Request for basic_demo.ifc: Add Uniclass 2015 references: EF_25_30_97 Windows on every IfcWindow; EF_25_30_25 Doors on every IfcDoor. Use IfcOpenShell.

First a look at what the model holds.

```python
import ifcopenshell

model = ifcopenshell.open("basic_demo.ifc")
print(model.schema)
print("classifications:", [c.Name for c in model.by_type("IfcClassification")])
for ifc_class in ("IfcDoor", "IfcRoof", "IfcStair", "IfcWall", "IfcWindow"):
    print(ifc_class, len(model.by_type(ifc_class)))
```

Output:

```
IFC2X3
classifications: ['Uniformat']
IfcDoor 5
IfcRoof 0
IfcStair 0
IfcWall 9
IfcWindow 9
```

```python
import ifcopenshell
import ifcopenshell.api.classification

model = ifcopenshell.open("basic_demo.ifc")

# IFC2X3 requires Source and Edition and has no link from the project to the system.
system = model.create_entity("IfcClassification", Source="NBS", Edition="2015", Name="Uniclass 2015")

codes = {
    "IfcWindow": ("EF_25_30_97", "Windows"),
    "IfcDoor": ("EF_25_30_25", "Doors"),
}
for ifc_class, (code, name) in codes.items():
    products = model.by_type(ifc_class)
    ifcopenshell.api.classification.add_reference(
        model, products=products, classification=system, identification=code, name=name
    )
    print(code, len(products))

model.write("basic_demo_updated.ifc")
```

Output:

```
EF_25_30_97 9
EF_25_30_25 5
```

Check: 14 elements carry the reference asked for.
